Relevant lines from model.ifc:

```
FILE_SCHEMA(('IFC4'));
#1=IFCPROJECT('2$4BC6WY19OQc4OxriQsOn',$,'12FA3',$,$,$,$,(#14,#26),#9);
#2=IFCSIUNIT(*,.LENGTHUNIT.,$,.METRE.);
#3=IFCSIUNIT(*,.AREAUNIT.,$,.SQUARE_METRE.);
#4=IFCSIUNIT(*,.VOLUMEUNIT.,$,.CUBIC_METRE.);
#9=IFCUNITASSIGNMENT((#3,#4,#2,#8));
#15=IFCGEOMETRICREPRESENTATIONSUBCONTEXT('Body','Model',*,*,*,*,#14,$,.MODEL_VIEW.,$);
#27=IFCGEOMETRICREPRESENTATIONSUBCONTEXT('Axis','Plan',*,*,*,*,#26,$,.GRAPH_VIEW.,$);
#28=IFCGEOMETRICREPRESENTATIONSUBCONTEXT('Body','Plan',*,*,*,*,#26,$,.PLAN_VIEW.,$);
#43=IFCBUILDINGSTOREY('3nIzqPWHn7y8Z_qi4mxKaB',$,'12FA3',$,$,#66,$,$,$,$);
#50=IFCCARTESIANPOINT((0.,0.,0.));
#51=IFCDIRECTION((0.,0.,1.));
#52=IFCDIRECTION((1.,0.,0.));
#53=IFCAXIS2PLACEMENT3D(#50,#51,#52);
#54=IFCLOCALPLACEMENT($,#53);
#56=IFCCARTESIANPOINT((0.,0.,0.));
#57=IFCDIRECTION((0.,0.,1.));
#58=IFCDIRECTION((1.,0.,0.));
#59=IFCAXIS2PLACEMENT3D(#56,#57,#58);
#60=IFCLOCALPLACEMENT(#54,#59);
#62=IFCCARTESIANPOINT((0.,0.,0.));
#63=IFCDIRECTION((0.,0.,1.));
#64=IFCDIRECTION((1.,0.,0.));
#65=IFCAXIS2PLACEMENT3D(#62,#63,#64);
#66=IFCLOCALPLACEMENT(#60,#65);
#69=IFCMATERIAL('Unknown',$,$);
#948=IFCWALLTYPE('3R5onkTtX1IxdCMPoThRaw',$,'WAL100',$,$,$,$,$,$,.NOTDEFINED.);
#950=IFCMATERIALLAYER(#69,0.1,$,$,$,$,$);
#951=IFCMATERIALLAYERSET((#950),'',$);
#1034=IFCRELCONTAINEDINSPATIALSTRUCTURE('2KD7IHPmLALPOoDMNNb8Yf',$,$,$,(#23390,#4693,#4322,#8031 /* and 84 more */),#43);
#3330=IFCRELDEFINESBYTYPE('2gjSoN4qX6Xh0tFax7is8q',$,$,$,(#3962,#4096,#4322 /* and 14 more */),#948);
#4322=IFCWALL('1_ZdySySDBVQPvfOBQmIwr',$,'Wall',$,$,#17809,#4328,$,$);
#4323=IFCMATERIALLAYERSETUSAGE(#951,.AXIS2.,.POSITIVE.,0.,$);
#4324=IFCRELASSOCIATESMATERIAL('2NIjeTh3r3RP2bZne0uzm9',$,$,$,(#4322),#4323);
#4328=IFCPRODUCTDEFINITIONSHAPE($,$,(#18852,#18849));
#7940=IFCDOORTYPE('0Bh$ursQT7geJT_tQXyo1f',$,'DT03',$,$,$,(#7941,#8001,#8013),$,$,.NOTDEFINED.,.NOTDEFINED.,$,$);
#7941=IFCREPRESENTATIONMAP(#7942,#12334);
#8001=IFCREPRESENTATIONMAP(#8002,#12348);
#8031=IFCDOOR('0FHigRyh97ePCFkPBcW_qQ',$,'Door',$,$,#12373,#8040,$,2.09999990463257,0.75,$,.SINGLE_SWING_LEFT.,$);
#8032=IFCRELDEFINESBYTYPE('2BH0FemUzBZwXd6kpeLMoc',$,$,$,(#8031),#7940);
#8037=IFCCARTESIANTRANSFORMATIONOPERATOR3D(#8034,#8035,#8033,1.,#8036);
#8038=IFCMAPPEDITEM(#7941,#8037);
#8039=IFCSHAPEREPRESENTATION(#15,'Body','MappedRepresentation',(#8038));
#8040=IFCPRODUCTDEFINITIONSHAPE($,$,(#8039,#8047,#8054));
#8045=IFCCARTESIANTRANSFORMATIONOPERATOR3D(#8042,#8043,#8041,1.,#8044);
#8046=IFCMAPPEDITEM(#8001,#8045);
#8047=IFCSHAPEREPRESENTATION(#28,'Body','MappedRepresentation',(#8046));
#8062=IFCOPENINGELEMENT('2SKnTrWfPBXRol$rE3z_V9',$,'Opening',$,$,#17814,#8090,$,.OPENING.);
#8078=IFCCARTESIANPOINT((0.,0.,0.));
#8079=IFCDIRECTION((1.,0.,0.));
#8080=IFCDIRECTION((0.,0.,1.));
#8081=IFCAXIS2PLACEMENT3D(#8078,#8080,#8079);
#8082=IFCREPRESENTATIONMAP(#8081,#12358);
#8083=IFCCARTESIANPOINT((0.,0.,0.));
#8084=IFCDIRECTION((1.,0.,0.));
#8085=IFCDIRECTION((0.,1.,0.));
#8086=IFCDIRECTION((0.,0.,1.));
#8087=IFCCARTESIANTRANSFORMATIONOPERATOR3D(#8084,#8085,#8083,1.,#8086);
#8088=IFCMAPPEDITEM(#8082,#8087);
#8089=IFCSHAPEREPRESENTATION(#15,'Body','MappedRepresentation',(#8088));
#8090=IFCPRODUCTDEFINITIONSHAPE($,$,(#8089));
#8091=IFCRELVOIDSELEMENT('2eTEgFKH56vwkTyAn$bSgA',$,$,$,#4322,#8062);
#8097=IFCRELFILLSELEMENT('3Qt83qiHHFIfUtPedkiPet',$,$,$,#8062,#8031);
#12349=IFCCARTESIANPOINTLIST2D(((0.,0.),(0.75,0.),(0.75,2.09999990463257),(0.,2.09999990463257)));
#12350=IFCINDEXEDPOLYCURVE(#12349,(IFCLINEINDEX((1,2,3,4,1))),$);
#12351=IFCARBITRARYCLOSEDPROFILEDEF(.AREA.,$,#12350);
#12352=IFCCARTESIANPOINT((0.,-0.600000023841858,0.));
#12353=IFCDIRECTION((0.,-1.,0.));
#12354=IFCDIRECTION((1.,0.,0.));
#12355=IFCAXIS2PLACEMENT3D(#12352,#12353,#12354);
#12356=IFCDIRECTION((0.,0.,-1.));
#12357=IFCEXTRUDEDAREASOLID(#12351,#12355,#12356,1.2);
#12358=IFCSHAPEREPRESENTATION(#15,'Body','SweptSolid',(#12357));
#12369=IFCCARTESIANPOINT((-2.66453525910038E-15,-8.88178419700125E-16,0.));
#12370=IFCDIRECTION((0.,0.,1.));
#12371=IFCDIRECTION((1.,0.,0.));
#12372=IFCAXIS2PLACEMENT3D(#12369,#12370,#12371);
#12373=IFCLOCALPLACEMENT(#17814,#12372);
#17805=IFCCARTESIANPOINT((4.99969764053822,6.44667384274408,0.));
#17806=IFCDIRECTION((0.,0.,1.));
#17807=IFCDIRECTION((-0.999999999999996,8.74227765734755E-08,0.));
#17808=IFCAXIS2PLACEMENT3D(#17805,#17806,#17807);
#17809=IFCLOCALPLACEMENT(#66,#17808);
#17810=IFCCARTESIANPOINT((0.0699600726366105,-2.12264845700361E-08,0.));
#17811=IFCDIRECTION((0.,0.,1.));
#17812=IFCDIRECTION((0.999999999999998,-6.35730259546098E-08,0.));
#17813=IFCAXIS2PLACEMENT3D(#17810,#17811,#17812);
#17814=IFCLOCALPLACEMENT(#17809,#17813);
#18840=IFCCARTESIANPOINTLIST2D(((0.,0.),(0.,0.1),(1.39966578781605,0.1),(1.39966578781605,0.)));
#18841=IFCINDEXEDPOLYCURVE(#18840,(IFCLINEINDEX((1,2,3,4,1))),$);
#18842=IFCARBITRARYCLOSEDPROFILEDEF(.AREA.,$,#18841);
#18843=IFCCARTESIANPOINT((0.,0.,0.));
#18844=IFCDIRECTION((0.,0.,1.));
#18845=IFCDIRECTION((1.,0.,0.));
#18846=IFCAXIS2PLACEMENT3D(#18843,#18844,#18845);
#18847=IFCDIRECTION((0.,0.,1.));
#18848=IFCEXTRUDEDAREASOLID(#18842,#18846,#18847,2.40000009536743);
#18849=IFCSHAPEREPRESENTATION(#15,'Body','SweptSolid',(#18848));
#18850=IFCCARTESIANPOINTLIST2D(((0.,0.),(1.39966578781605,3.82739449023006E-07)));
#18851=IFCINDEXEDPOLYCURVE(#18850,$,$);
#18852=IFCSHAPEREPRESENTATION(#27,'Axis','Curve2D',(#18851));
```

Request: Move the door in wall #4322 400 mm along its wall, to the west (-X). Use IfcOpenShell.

```python
import ifcopenshell
import ifcopenshell.api.geometry
import ifcopenshell.util.placement
import ifcopenshell.util.unit

model = ifcopenshell.open("model.ifc")
unit_scale = ifcopenshell.util.unit.calculate_unit_scale(model)

door = model.by_guid("0FHigRyh97ePCFkPBcW_qQ")
opening = door.FillsVoids[0].RelatingOpeningElement
wall = opening.VoidsElements[0].RelatingBuildingElement

wall_matrix = ifcopenshell.util.placement.get_local_placement(wall.ObjectPlacement)
shift = wall_matrix[:3, 0] * 0.4 / unit_scale
before = ifcopenshell.util.placement.get_local_placement(door.ObjectPlacement)[:3, 3].copy()

# The door is placed relative to its opening, so it follows when the opening moves.
matrix = ifcopenshell.util.placement.get_local_placement(opening.ObjectPlacement)
matrix[:3, 3] += shift
ifcopenshell.api.geometry.edit_object_placement(
    model, product=opening, matrix=matrix, is_si=False, should_transform_children=True
)

after = ifcopenshell.util.placement.get_local_placement(door.ObjectPlacement)[:3, 3]
print("door moved by", (after - before).round(3) + 0.0)

model.write("model_edited.ifc")
```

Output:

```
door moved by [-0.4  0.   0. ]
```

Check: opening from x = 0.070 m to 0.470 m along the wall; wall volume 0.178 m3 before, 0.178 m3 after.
